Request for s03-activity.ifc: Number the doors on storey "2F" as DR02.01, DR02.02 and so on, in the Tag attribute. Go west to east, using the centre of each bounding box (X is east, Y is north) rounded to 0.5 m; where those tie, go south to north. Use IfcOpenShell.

First a look at what the model holds.

```python
import ifcopenshell
import ifcopenshell.util.element
import ifcopenshell.util.placement

model = ifcopenshell.open("s03-activity.ifc")
print(model.schema)
storey = next(s for s in model.by_type("IfcBuildingStorey") if s.Name == "2F")
doors = [e for e in ifcopenshell.util.element.get_decomposition(storey) if e.is_a("IfcDoor")]
for e in sorted(doors, key=lambda e: e.id()):
    origin = ifcopenshell.util.placement.get_local_placement(e.ObjectPlacement)[:3, 3]
    print(e.id(), e.Tag, e.Name, origin.round(2) + 0.0, sep=" | ")
```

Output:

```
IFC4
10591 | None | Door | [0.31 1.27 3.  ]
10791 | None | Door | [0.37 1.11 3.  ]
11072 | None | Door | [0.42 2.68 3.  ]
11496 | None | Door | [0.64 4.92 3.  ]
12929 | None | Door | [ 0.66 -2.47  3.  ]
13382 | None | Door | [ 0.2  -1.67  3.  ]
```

```python
import ifcopenshell
import ifcopenshell.geom
import ifcopenshell.util.element
import ifcopenshell.util.shape

model = ifcopenshell.open("s03-activity.ifc")
settings = ifcopenshell.geom.settings()
settings.set("use-world-coords", True)


def centre(element):
    shape = ifcopenshell.geom.create_shape(settings, element)
    return ifcopenshell.util.shape.get_bbox_centroid(shape.geometry)


storey = next(s for s in model.by_type("IfcBuildingStorey") if s.Name == "2F")
doors = [e for e in ifcopenshell.util.element.get_decomposition(storey) if e.is_a("IfcDoor")]

# Insertion points can sit at a corner or the storey origin, so sort by the geometry (in metres).
centres = {e: centre(e) for e in doors}
doors.sort(key=lambda e: (round(centres[e][0] / 0.5), centres[e][1]))

for i, e in enumerate(doors, start=1):
    number = f"DR02.{i:02d}"
    e.Tag = number
    print(e.id(), number)

model.write("s03-activity_rev.ifc")
```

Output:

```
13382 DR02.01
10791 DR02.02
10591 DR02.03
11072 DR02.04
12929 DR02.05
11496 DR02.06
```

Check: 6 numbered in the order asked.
